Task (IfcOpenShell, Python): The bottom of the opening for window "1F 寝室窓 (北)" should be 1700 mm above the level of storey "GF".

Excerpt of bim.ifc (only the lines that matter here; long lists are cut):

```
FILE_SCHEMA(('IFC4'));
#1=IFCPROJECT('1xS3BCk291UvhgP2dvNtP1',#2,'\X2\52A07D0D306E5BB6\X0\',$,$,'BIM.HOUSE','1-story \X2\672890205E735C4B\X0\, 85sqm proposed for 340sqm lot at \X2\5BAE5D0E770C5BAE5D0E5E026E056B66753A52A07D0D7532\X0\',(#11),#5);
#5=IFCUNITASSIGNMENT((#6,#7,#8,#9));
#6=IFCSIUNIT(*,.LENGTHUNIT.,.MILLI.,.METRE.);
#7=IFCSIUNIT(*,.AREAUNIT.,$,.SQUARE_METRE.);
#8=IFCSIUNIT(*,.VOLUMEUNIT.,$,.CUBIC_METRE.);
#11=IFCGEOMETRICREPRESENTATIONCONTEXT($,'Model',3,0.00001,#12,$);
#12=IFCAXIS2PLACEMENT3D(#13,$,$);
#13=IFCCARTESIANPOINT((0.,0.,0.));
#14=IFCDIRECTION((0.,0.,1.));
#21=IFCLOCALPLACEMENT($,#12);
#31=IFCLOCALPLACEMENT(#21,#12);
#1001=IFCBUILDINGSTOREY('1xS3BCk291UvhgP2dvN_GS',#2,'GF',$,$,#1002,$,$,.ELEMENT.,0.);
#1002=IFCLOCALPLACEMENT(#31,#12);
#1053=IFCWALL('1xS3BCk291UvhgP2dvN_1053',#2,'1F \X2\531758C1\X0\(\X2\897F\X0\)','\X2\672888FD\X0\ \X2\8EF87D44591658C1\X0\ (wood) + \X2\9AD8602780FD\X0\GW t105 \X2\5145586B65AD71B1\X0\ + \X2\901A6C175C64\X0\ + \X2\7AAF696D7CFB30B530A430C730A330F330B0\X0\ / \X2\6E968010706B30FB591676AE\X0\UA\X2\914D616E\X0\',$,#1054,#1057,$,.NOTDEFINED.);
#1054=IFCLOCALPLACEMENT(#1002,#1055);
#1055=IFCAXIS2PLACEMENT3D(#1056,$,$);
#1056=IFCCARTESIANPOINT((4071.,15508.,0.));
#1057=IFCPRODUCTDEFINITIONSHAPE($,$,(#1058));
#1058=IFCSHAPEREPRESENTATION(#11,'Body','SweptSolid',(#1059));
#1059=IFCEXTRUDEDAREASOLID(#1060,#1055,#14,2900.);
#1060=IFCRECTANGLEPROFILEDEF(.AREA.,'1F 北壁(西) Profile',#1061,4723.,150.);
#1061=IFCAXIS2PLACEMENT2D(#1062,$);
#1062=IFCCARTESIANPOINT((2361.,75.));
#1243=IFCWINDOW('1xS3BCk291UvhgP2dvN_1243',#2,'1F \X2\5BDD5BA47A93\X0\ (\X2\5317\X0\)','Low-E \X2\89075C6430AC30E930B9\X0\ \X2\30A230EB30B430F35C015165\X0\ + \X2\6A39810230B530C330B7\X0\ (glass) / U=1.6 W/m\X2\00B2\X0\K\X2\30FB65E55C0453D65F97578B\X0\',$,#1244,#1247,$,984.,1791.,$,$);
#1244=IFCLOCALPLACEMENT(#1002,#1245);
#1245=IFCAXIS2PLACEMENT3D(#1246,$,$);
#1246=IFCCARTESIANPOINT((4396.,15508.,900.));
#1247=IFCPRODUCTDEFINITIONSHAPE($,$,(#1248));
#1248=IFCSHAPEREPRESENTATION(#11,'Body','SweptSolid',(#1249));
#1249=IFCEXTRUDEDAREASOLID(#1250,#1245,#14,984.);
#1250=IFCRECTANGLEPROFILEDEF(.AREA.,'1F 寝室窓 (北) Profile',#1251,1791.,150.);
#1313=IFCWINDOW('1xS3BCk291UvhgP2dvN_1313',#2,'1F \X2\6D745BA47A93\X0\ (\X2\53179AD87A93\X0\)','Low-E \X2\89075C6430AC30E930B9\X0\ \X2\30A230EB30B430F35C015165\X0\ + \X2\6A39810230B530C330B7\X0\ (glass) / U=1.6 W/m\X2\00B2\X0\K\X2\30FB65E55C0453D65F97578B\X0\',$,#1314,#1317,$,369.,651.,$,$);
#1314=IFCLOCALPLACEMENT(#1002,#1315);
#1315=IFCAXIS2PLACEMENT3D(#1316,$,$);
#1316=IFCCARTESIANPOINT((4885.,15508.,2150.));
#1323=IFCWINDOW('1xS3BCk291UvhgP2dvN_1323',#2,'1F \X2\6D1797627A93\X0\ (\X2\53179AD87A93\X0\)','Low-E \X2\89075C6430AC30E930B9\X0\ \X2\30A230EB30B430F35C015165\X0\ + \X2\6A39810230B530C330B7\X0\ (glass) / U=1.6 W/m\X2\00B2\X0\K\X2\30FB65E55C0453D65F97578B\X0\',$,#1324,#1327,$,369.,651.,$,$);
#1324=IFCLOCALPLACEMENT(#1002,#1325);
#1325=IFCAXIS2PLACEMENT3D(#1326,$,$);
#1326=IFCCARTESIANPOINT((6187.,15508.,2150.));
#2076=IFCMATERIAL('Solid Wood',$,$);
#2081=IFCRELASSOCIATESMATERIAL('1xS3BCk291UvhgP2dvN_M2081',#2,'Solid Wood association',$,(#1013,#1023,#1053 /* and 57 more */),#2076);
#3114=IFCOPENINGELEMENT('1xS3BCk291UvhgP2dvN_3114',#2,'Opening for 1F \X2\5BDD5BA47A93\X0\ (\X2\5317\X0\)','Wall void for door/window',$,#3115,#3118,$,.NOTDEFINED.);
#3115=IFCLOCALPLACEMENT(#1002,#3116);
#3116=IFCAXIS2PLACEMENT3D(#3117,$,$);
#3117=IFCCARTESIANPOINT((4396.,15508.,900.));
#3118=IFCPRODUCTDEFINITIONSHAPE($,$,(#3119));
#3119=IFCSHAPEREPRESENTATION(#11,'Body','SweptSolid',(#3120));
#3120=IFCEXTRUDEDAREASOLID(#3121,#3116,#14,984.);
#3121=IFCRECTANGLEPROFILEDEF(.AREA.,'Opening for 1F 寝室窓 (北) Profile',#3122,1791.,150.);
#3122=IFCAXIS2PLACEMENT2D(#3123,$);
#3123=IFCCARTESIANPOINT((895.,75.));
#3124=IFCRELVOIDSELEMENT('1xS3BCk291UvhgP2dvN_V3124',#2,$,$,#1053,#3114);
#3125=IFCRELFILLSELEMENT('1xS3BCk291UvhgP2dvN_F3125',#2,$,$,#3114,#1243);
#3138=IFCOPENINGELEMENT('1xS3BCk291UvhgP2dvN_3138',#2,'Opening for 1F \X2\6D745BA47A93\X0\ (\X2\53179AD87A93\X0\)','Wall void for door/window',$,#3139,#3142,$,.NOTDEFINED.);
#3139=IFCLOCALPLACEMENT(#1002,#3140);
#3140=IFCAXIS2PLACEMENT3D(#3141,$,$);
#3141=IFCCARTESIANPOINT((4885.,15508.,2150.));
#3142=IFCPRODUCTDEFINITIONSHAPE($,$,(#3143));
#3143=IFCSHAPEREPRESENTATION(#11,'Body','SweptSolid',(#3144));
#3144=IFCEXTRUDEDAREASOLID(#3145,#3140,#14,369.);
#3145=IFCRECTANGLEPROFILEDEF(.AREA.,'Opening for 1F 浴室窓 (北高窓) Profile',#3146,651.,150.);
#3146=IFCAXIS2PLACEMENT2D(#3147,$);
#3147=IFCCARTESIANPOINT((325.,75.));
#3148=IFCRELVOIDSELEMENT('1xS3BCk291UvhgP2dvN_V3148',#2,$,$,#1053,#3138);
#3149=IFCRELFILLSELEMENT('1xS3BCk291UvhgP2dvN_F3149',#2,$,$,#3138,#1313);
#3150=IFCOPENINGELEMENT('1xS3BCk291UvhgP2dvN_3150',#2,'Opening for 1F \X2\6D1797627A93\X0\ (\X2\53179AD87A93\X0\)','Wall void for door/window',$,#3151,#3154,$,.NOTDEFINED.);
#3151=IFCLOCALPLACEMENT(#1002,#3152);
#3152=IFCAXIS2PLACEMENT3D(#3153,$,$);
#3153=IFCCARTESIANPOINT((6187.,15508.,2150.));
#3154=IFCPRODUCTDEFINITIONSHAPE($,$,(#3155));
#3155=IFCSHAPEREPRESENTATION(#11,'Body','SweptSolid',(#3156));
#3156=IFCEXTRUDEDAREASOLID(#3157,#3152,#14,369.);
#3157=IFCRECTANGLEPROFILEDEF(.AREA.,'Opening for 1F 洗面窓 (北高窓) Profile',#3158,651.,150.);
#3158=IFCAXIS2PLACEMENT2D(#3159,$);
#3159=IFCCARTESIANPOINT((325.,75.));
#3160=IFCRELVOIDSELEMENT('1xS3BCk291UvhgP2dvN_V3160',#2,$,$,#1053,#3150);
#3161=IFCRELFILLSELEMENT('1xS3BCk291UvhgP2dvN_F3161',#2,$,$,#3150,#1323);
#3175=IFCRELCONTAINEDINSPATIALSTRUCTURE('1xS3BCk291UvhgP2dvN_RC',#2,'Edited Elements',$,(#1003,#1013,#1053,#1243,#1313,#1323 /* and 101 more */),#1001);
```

```python
import numpy as np
import ifcopenshell
import ifcopenshell.api.geometry
import ifcopenshell.geom
import ifcopenshell.util.element
import ifcopenshell.util.placement
import ifcopenshell.util.shape
import ifcopenshell.util.unit

model = ifcopenshell.open("bim.ifc")
unit_scale = ifcopenshell.util.unit.calculate_unit_scale(model)

window = model.by_id(1243)
opening = window.FillsVoids[0].RelatingOpeningElement
storey = ifcopenshell.util.element.get_container(window, ifc_class="IfcBuildingStorey")
level = ifcopenshell.util.placement.get_local_placement(storey.ObjectPlacement)[2, 3]

# The opening's origin need not be at the sill, so measure its lowest point.
shape = ifcopenshell.geom.create_shape(ifcopenshell.geom.settings(), opening)
bottom = ifcopenshell.util.shape.get_shape_bottom_elevation(shape, shape.geometry) / unit_scale
dz = level + 1.7 / unit_scale - bottom

shift = np.array([0.0, 0.0, dz])
# The window is not placed relative to its opening, so move both.
for product in (opening, window):
    matrix = ifcopenshell.util.placement.get_local_placement(product.ObjectPlacement)
    matrix[:3, 3] += shift
    ifcopenshell.api.geometry.edit_object_placement(model, product=product, matrix=matrix, is_si=False)

print(f"moved by {dz * unit_scale:+.3f} m")

model.write("bim-out.ifc")
```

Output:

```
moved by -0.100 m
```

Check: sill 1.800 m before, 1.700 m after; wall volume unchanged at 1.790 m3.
